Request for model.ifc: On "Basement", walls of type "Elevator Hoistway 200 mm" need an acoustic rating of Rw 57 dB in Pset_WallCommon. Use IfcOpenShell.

First a look at what the model holds.

```python
import ifcopenshell
import ifcopenshell.util.element

model = ifcopenshell.open("model.ifc")
print(model.schema)
storey = next(s for s in model.by_type("IfcBuildingStorey") if s.Name == "Basement")
walls = [e for e in ifcopenshell.util.element.get_decomposition(storey) if e.is_a("IfcWall")]
seen = {}
for e in walls:
    element_type = ifcopenshell.util.element.get_type(e)
    key = (element_type.Name if element_type != e and element_type else None, ifcopenshell.util.element.get_pset(e, "Pset_WallCommon", "AcousticRating"))
    seen[key] = seen.get(key, 0) + 1
for (name, value), count in sorted(seen.items(), key=str):
    print(count, "x", name, "|", value)
```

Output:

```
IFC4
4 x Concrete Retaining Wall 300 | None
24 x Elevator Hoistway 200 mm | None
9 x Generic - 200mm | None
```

```python
import ifcopenshell
import ifcopenshell.api.pset
import ifcopenshell.util.element

model = ifcopenshell.open("model.ifc")

storey = next(s for s in model.by_type("IfcBuildingStorey") if s.Name == "Basement")
walls = [e for e in ifcopenshell.util.element.get_decomposition(storey) if e.is_a("IfcWall")]

count = 0
for e in walls:
    element_type = ifcopenshell.util.element.get_type(e)
    if element_type in (None, e) or element_type.Name != "Elevator Hoistway 200 mm":
        continue
    # add_pset returns the element's existing set when there is one.
    pset = ifcopenshell.api.pset.add_pset(model, product=e, name="Pset_WallCommon")
    ifcopenshell.api.pset.edit_pset(model, pset=pset, properties={"AcousticRating": "Rw 57 dB"})
    count += 1

print(count, "walls updated")

model.write("model_rev.ifc")
```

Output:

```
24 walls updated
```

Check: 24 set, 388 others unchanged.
